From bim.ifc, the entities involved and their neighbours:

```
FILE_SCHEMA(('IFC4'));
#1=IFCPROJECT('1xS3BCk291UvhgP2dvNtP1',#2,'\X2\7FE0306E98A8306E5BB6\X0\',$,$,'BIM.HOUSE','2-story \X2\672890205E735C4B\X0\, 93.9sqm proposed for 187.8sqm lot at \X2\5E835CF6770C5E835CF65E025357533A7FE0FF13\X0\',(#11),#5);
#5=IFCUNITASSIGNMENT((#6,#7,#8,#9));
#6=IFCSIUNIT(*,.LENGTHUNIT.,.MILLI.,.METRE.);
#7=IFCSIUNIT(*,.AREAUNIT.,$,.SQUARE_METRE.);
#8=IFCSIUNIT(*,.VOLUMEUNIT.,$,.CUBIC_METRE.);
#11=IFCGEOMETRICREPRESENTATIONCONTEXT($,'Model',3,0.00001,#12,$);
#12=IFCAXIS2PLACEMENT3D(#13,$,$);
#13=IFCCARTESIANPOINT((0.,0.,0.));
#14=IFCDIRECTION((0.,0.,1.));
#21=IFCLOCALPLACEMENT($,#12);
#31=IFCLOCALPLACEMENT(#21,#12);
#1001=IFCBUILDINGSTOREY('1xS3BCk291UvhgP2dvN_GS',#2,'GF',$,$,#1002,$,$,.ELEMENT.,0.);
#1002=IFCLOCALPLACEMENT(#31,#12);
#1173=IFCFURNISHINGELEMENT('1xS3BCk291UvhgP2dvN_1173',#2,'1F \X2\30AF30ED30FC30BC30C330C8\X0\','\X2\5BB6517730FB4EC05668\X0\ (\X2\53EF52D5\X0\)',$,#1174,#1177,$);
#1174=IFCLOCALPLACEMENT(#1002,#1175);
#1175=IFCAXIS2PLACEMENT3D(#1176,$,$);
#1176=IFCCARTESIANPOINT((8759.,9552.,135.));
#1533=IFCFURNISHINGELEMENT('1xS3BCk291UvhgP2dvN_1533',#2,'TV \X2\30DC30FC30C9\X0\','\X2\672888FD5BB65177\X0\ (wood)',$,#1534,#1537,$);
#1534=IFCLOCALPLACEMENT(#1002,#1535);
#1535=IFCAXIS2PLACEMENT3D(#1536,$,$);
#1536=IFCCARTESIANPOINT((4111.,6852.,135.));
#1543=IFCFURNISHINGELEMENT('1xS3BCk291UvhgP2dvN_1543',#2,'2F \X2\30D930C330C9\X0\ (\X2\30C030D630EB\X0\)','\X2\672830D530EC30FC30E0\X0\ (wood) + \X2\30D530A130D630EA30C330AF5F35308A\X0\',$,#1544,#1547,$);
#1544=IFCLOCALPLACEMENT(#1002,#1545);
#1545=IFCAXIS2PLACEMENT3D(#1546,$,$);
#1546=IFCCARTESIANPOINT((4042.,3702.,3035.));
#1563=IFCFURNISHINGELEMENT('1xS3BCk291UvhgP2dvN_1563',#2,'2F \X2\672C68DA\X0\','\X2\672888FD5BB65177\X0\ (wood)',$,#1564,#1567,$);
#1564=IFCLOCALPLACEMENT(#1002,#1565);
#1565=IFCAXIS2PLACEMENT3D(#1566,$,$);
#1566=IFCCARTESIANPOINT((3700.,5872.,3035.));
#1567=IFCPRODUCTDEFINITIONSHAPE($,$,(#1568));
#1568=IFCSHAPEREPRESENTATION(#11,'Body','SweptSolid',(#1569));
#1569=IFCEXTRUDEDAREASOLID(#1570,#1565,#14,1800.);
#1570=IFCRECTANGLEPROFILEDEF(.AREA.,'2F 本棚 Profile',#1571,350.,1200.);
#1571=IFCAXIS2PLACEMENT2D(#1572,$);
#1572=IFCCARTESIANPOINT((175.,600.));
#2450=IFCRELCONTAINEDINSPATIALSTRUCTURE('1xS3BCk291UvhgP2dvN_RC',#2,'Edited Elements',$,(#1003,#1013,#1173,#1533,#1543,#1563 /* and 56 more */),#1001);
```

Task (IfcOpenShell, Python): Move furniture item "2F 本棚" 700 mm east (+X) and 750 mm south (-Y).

```python
import ifcopenshell
import ifcopenshell.api.geometry
import ifcopenshell.util.placement
import ifcopenshell.util.unit

model = ifcopenshell.open("bim.ifc")
unit_scale = ifcopenshell.util.unit.calculate_unit_scale(model)

item = model.by_id(1563)
matrix = ifcopenshell.util.placement.get_local_placement(item.ObjectPlacement)
matrix[0, 3] += 0.7 / unit_scale
matrix[1, 3] -= 0.75 / unit_scale
ifcopenshell.api.geometry.edit_object_placement(model, product=item, matrix=matrix, is_si=False)

print(ifcopenshell.util.placement.get_local_placement(item.ObjectPlacement).round(3) + 0.0)

model.write("bim_edited.ifc")
```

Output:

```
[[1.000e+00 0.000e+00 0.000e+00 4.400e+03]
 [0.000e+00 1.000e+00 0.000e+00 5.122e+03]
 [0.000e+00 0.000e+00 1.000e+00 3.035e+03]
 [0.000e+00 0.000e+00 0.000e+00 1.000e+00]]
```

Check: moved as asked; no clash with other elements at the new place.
